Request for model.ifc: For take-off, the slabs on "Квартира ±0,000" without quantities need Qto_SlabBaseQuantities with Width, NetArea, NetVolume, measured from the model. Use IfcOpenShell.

First a look at what the model holds.

```python
import ifcopenshell
import ifcopenshell.util.element
import ifcopenshell.util.unit

model = ifcopenshell.open("model.ifc")
print(model.schema)
for unit_type in ("LENGTHUNIT", "AREAUNIT", "VOLUMEUNIT"):
    print(unit_type, ifcopenshell.util.unit.calculate_unit_scale(model, unit_type))
storey = next(s for s in model.by_type("IfcBuildingStorey") if s.Name == "Квартира ±0,000")
slabs = [e for e in ifcopenshell.util.element.get_decomposition(storey) if e.is_a("IfcSlab")]
for e in sorted(slabs, key=lambda e: e.id()):
    print(e.id(), e.is_a(), e.Name, list(ifcopenshell.util.element.get_psets(e, qtos_only=True)), sep=" | ")
```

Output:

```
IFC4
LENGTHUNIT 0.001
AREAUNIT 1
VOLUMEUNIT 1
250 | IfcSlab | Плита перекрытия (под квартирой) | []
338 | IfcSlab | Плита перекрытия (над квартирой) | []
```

```python
import ifcopenshell
import ifcopenshell.api.pset
import ifcopenshell.geom
import ifcopenshell.util.element
import ifcopenshell.util.shape
import ifcopenshell.util.unit

model = ifcopenshell.open("model.ifc")
unit_scale = ifcopenshell.util.unit.calculate_unit_scale(model)
area_scale = ifcopenshell.util.unit.calculate_unit_scale(model, "AREAUNIT")
volume_scale = ifcopenshell.util.unit.calculate_unit_scale(model, "VOLUMEUNIT")
settings = ifcopenshell.geom.settings()

storey = next(s for s in model.by_type("IfcBuildingStorey") if s.Name == "Квартира ±0,000")
slabs = [e for e in ifcopenshell.util.element.get_decomposition(storey) if e.is_a("IfcSlab")]

for e in sorted(slabs, key=lambda e: e.id()):
    if ifcopenshell.util.element.get_psets(e, qtos_only=True, should_inherit=False):
        continue
    # Geometry comes back in metres, in the element's own axes.
    shape = ifcopenshell.geom.create_shape(settings, e)
    values = {
        "Width": ifcopenshell.util.shape.get_z(shape.geometry) / unit_scale,
        "NetArea": ifcopenshell.util.shape.get_footprint_area(shape.geometry) / area_scale,
        "NetVolume": ifcopenshell.util.shape.get_volume(shape.geometry) / volume_scale,
    }
    qto = ifcopenshell.api.pset.add_qto(model, product=e, name="Qto_SlabBaseQuantities")
    ifcopenshell.api.pset.edit_qto(model, qto=qto, properties=values)
    print(e.id(), {k: round(v, 3) for k, v in values.items()})

model.write("model_v2.ifc")
```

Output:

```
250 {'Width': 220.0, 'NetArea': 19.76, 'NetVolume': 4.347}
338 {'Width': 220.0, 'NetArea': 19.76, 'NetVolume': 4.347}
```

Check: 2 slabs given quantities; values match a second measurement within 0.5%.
